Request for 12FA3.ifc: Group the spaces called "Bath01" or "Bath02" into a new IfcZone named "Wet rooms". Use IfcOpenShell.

First a look at what the model holds.

```python
import ifcopenshell

model = ifcopenshell.open("12FA3.ifc")
print(model.schema)
seen = {}
for space in model.by_type("IfcSpace"):
    seen[space.Name] = seen.get(space.Name, 0) + 1
for name, count in sorted(seen.items(), key=str):
    print(count, "x", name)
print("zones:", [z.Name for z in model.by_type("IfcZone")][:20])
```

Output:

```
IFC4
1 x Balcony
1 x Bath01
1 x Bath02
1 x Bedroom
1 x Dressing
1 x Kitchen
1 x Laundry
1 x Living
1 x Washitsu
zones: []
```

```python
import ifcopenshell
import ifcopenshell.api.group
import ifcopenshell.api.root

model = ifcopenshell.open("12FA3.ifc")

names = {"Bath01", "Bath02"}
spaces = [s for s in model.by_type("IfcSpace") if s.Name in names]

zone = ifcopenshell.api.root.create_entity(model, ifc_class="IfcZone", name="Wet rooms")
ifcopenshell.api.group.assign_group(model, products=spaces, group=zone)
print(len(spaces), "spaces in", zone.Name)

model.write("12FA3-out.ifc")
```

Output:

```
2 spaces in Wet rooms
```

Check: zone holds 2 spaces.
